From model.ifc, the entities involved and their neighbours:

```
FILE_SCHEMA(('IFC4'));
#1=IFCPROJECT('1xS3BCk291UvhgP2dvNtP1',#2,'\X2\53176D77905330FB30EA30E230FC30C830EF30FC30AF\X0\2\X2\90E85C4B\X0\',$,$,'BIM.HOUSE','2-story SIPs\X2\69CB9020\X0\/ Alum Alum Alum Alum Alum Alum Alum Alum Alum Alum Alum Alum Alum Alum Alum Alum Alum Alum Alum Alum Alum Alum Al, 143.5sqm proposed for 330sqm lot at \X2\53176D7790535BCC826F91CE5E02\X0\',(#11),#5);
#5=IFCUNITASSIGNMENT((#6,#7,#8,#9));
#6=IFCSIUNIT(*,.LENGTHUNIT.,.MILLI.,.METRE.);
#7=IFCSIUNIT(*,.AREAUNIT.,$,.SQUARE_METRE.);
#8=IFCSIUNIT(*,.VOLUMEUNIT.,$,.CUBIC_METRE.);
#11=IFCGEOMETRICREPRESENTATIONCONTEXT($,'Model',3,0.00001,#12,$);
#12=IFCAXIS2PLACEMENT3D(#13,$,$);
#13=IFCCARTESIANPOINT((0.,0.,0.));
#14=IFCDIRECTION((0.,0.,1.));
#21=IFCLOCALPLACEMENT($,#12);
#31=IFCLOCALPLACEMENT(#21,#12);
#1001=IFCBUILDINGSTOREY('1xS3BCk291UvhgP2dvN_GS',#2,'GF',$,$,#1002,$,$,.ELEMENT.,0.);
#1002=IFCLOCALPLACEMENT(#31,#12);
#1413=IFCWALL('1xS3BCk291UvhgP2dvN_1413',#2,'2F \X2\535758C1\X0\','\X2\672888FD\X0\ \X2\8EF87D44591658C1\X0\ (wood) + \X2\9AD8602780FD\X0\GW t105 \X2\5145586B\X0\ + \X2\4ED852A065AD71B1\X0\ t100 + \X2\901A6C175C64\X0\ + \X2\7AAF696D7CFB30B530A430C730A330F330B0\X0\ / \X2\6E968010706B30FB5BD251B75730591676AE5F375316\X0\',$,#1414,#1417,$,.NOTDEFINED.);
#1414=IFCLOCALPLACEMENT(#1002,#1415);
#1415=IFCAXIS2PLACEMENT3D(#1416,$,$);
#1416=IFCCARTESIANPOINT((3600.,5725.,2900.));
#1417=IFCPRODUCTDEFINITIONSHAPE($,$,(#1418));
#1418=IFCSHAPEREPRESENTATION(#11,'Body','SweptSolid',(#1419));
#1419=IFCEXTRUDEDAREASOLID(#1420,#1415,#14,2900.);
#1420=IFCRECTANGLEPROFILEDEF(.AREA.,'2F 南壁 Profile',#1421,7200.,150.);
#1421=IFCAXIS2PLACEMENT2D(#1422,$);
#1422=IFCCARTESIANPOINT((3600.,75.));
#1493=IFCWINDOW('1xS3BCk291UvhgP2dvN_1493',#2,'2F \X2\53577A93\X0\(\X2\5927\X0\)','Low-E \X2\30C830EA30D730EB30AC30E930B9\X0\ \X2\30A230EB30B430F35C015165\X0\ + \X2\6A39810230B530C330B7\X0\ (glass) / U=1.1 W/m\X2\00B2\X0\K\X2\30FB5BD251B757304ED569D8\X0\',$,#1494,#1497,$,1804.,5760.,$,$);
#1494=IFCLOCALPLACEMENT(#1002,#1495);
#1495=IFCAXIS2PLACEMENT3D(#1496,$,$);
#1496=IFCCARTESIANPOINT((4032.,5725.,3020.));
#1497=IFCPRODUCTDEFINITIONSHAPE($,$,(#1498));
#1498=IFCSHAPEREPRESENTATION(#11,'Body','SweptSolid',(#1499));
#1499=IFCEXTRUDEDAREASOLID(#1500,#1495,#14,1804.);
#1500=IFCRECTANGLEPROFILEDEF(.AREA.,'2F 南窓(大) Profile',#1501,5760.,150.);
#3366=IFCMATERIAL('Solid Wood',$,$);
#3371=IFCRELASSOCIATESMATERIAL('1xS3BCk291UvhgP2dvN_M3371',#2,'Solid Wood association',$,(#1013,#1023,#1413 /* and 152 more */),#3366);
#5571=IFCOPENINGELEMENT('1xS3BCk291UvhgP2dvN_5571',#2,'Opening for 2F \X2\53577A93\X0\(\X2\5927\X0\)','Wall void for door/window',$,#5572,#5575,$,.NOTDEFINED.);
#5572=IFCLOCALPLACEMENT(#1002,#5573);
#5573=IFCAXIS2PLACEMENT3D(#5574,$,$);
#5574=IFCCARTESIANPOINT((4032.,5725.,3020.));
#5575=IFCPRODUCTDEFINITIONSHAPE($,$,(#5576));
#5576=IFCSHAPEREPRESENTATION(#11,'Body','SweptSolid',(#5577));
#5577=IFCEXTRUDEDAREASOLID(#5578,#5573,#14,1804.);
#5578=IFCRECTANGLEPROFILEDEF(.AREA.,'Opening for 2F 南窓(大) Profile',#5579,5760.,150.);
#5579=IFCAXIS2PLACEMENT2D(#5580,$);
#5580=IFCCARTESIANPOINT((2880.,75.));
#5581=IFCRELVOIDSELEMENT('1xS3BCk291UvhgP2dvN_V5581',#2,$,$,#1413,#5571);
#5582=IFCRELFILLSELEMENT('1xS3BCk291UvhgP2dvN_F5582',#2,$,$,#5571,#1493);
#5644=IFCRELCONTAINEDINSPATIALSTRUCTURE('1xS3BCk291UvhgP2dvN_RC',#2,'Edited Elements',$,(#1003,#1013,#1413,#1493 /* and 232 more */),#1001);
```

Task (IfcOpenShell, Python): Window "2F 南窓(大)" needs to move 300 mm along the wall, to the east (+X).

```python
import ifcopenshell
import ifcopenshell.api.geometry
import ifcopenshell.util.placement
import ifcopenshell.util.unit

model = ifcopenshell.open("model.ifc")
unit_scale = ifcopenshell.util.unit.calculate_unit_scale(model)

window = model.by_guid("1xS3BCk291UvhgP2dvN_1493")
opening = window.FillsVoids[0].RelatingOpeningElement
wall = opening.VoidsElements[0].RelatingBuildingElement

wall_matrix = ifcopenshell.util.placement.get_local_placement(wall.ObjectPlacement)
shift = wall_matrix[:3, 0] * 0.3 / unit_scale
before = ifcopenshell.util.placement.get_local_placement(window.ObjectPlacement)[:3, 3].copy()

# The window is not placed relative to its opening, so move both.
for product in (opening, window):
    matrix = ifcopenshell.util.placement.get_local_placement(product.ObjectPlacement)
    matrix[:3, 3] += shift
    ifcopenshell.api.geometry.edit_object_placement(model, product=product, matrix=matrix, is_si=False)

after = ifcopenshell.util.placement.get_local_placement(window.ObjectPlacement)[:3, 3]
print("window moved by", (after - before).round(3) + 0.0)

model.write("model_edited.ifc")
```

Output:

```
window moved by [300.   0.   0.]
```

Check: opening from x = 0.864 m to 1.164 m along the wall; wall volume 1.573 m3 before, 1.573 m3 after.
